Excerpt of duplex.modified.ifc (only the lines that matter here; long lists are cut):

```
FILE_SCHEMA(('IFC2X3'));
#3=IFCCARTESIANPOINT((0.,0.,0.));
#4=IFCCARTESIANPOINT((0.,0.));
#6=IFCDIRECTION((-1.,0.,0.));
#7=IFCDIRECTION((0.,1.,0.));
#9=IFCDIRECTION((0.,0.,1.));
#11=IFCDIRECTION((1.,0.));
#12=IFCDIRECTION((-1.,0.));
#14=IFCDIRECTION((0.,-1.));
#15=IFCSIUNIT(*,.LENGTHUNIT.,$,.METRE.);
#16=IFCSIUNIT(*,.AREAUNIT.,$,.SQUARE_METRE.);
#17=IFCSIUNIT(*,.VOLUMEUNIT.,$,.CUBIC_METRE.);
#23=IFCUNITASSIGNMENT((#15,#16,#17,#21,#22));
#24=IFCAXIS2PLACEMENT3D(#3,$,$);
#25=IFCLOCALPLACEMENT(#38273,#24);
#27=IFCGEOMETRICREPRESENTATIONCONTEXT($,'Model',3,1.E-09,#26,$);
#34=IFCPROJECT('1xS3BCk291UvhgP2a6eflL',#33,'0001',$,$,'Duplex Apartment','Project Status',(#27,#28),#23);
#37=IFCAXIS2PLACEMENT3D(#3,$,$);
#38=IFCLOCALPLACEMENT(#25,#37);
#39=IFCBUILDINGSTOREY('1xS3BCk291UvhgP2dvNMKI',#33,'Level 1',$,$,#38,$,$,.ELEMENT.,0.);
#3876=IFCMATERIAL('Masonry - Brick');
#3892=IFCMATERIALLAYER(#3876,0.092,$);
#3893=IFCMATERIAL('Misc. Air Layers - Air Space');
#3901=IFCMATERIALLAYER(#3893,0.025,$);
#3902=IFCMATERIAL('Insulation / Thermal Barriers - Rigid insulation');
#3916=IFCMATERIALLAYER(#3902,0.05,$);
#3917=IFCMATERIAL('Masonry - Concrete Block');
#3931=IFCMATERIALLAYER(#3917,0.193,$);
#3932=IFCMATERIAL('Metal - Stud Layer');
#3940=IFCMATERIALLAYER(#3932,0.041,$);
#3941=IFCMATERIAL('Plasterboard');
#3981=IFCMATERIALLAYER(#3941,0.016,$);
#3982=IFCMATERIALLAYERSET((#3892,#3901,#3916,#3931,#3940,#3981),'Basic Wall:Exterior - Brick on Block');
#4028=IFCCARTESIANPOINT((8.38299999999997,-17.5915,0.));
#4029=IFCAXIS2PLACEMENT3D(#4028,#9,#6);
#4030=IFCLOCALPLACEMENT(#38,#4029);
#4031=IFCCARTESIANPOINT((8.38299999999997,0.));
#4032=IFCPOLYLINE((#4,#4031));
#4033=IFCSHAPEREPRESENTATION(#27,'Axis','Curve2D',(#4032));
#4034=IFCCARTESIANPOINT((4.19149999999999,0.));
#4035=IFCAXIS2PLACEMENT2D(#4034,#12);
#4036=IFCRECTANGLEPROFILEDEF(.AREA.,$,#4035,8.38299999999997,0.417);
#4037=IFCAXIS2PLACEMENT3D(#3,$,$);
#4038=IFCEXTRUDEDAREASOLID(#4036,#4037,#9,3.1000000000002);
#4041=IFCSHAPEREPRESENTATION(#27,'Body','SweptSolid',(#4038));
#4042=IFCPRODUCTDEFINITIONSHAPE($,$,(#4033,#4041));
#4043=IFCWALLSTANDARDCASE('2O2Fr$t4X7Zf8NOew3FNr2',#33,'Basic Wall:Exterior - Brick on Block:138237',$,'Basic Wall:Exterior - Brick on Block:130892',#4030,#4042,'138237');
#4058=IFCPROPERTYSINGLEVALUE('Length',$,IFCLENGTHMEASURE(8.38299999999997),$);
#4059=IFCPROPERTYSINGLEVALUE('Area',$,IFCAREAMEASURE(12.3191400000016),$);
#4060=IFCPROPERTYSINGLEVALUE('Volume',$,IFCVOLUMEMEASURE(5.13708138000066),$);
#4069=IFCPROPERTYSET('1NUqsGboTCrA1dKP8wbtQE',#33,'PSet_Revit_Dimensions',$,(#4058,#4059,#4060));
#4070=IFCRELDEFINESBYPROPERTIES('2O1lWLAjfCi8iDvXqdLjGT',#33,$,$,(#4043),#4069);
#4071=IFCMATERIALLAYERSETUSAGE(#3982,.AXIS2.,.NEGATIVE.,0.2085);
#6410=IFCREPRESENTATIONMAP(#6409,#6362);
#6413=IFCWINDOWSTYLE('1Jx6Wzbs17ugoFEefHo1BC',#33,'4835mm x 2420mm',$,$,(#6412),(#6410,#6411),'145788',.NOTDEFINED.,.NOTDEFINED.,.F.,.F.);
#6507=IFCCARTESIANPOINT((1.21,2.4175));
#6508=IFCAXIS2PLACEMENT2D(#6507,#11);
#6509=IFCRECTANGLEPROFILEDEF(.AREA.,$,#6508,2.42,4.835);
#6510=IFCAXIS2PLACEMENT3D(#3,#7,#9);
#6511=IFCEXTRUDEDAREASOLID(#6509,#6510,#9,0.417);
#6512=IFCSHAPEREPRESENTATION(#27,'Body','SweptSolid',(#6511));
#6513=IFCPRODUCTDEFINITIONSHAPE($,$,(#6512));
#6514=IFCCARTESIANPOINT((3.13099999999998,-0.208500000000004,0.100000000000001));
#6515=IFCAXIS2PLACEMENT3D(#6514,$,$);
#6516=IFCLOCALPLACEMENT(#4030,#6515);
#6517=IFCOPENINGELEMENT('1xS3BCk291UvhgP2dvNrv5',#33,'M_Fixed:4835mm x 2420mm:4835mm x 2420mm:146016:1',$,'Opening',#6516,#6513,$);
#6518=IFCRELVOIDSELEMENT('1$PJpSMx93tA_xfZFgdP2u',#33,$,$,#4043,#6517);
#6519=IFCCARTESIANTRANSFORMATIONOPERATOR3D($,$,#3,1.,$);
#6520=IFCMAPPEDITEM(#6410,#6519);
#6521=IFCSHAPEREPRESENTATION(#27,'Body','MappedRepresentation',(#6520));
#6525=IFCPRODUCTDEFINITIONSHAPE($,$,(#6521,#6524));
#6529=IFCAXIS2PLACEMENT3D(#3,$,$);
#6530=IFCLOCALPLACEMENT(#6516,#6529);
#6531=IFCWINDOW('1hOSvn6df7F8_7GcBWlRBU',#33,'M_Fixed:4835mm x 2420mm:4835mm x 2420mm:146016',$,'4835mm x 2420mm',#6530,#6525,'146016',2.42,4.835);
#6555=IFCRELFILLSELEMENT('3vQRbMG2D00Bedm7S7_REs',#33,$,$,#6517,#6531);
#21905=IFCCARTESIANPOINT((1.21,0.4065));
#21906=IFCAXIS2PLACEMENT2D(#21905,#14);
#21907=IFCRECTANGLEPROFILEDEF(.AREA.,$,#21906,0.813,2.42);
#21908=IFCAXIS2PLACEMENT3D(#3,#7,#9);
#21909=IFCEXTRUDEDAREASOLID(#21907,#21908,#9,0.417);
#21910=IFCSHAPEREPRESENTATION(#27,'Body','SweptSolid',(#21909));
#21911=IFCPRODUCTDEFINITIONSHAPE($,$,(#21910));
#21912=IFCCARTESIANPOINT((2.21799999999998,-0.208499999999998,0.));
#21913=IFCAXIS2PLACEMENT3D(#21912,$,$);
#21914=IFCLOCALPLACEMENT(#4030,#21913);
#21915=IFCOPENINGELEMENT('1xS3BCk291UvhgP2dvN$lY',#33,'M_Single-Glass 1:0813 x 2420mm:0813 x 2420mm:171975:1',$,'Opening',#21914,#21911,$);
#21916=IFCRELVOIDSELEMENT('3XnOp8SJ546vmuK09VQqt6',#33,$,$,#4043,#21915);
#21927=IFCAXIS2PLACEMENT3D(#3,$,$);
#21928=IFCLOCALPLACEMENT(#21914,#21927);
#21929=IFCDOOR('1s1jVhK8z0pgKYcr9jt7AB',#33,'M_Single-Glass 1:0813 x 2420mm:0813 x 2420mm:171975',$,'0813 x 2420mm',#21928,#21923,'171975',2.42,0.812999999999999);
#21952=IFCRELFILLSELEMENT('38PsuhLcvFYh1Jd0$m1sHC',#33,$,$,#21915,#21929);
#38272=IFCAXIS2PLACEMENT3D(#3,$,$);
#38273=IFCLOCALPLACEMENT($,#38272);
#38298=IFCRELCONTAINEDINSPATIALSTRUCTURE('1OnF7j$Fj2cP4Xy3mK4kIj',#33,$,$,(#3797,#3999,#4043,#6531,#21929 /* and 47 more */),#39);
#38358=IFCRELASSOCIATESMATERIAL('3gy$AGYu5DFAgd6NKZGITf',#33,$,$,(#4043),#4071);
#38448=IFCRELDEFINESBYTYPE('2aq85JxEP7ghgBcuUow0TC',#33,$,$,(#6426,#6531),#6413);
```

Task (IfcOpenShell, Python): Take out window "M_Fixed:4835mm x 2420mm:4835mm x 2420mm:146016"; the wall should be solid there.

```python
import ifcopenshell
import ifcopenshell.api.feature
import ifcopenshell.api.pset
import ifcopenshell.api.root
import ifcopenshell.geom
import ifcopenshell.util.element
import ifcopenshell.util.shape
import ifcopenshell.util.unit

model = ifcopenshell.open("duplex.modified.ifc")
area_scale = ifcopenshell.util.unit.calculate_unit_scale(model, "AREAUNIT")
volume_scale = ifcopenshell.util.unit.calculate_unit_scale(model, "VOLUMEUNIT")
settings = ifcopenshell.geom.settings()


def volume(element):
    """Net volume in cubic metres, openings subtracted."""
    shape = ifcopenshell.geom.create_shape(settings, element)
    return ifcopenshell.util.shape.get_volume(shape.geometry)


window = model.by_guid("1hOSvn6df7F8_7GcBWlRBU")
opening = window.FillsVoids[0].RelatingOpeningElement
wall = opening.VoidsElements[0].RelatingBuildingElement
before = volume(wall)

ifcopenshell.api.root.remove_product(model, product=window)
ifcopenshell.api.feature.remove_feature(model, feature=opening)

after = volume(wall)
thickness = 0.417  # wall thickness in metres

# Update the wall's stored quantities.
pset = model.by_id(ifcopenshell.util.element.get_pset(wall, "PSet_Revit_Dimensions", should_inherit=False)["id"])
ifcopenshell.api.pset.edit_pset(model, pset=pset, properties={
    "Area": model.create_entity("IfcAreaMeasure", after / thickness / area_scale),
    "Volume": model.create_entity("IfcVolumeMeasure", after / volume_scale),
})

print(f"wall volume {before:.3f} -> {after:.3f} m3")

model.write("duplex.modified_updated.ifc")
```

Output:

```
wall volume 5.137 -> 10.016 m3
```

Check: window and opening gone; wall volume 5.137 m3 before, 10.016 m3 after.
